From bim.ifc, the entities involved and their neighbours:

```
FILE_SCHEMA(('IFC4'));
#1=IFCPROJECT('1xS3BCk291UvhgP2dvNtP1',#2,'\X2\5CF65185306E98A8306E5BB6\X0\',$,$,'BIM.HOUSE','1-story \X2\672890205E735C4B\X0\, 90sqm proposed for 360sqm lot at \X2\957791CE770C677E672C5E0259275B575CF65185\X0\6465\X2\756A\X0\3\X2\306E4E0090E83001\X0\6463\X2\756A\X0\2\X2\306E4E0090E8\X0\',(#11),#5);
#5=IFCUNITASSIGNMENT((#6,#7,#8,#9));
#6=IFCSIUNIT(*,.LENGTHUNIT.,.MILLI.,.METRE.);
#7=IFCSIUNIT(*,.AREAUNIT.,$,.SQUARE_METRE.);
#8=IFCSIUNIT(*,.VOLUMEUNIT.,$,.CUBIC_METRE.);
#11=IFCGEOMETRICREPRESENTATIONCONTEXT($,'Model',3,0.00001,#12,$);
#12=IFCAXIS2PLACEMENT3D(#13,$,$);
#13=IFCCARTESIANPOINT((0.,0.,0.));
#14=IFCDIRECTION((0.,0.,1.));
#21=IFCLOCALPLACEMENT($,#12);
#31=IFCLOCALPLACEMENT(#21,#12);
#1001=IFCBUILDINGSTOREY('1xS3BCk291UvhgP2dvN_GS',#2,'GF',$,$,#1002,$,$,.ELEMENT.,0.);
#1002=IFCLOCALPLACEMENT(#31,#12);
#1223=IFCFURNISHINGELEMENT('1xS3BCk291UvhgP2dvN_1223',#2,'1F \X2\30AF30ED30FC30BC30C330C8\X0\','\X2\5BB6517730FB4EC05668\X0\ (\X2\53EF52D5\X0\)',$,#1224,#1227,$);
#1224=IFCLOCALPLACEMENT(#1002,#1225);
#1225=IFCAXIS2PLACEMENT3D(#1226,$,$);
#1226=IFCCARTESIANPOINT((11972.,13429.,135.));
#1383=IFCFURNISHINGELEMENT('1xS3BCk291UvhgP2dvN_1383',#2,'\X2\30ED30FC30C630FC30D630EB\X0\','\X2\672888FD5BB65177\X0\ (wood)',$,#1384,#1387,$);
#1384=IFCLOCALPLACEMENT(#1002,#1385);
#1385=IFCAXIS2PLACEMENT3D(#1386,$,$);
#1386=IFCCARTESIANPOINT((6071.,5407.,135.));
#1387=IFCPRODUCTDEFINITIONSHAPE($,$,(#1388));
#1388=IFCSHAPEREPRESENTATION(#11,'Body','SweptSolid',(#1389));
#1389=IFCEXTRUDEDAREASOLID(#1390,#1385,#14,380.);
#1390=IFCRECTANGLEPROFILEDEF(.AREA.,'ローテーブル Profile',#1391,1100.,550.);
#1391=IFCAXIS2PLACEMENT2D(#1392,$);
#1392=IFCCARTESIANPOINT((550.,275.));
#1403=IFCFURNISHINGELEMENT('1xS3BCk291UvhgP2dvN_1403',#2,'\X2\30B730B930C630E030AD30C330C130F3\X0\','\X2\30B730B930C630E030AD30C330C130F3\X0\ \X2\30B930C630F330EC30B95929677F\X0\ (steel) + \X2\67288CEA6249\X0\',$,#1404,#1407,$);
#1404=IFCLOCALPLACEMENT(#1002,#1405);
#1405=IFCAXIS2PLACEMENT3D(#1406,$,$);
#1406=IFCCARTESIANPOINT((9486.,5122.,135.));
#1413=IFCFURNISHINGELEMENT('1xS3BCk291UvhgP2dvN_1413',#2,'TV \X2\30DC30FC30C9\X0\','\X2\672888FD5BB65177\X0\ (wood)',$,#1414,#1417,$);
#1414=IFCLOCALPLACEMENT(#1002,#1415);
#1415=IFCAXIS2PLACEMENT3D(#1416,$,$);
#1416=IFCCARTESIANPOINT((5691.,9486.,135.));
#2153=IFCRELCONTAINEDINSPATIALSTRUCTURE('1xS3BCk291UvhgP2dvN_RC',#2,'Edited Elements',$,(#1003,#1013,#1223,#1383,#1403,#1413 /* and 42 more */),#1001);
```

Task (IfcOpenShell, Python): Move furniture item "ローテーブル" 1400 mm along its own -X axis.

```python
import ifcopenshell
import ifcopenshell.api.geometry
import ifcopenshell.util.placement
import ifcopenshell.util.unit

model = ifcopenshell.open("bim.ifc")
unit_scale = ifcopenshell.util.unit.calculate_unit_scale(model)

item = model.by_guid("1xS3BCk291UvhgP2dvN_1383")
matrix = ifcopenshell.util.placement.get_local_placement(item.ObjectPlacement)
matrix[:3, 3] -= matrix[:3, 0] * 1.4 / unit_scale
ifcopenshell.api.geometry.edit_object_placement(model, product=item, matrix=matrix, is_si=False)

print(ifcopenshell.util.placement.get_local_placement(item.ObjectPlacement).round(3) + 0.0)

model.write("bim_v2.ifc")
```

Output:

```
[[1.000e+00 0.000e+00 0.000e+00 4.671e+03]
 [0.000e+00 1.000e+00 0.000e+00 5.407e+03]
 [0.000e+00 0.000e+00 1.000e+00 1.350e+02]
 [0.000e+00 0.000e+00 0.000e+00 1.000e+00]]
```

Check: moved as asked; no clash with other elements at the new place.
